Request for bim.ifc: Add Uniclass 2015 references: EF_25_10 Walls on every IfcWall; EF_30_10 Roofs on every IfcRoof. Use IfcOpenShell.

First a look at what the model holds.

```python
import ifcopenshell

model = ifcopenshell.open("bim.ifc")
print(model.schema)
print("classifications:", [c.Name for c in model.by_type("IfcClassification")])
for ifc_class in ("IfcDoor", "IfcRoof", "IfcStair", "IfcWall", "IfcWindow"):
    print(ifc_class, len(model.by_type(ifc_class)))
```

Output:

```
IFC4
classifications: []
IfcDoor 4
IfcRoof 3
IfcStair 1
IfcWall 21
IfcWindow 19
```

```python
import ifcopenshell
import ifcopenshell.api.classification

model = ifcopenshell.open("bim.ifc")

system = ifcopenshell.api.classification.add_classification(model, classification="Uniclass 2015")

codes = {
    "IfcWall": ("EF_25_10", "Walls"),
    "IfcRoof": ("EF_30_10", "Roofs"),
}
for ifc_class, (code, name) in codes.items():
    products = model.by_type(ifc_class)
    ifcopenshell.api.classification.add_reference(
        model, products=products, classification=system, identification=code, name=name
    )
    print(code, len(products))

model.write("bim_v2.ifc")
```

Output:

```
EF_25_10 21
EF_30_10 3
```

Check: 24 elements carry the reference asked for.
